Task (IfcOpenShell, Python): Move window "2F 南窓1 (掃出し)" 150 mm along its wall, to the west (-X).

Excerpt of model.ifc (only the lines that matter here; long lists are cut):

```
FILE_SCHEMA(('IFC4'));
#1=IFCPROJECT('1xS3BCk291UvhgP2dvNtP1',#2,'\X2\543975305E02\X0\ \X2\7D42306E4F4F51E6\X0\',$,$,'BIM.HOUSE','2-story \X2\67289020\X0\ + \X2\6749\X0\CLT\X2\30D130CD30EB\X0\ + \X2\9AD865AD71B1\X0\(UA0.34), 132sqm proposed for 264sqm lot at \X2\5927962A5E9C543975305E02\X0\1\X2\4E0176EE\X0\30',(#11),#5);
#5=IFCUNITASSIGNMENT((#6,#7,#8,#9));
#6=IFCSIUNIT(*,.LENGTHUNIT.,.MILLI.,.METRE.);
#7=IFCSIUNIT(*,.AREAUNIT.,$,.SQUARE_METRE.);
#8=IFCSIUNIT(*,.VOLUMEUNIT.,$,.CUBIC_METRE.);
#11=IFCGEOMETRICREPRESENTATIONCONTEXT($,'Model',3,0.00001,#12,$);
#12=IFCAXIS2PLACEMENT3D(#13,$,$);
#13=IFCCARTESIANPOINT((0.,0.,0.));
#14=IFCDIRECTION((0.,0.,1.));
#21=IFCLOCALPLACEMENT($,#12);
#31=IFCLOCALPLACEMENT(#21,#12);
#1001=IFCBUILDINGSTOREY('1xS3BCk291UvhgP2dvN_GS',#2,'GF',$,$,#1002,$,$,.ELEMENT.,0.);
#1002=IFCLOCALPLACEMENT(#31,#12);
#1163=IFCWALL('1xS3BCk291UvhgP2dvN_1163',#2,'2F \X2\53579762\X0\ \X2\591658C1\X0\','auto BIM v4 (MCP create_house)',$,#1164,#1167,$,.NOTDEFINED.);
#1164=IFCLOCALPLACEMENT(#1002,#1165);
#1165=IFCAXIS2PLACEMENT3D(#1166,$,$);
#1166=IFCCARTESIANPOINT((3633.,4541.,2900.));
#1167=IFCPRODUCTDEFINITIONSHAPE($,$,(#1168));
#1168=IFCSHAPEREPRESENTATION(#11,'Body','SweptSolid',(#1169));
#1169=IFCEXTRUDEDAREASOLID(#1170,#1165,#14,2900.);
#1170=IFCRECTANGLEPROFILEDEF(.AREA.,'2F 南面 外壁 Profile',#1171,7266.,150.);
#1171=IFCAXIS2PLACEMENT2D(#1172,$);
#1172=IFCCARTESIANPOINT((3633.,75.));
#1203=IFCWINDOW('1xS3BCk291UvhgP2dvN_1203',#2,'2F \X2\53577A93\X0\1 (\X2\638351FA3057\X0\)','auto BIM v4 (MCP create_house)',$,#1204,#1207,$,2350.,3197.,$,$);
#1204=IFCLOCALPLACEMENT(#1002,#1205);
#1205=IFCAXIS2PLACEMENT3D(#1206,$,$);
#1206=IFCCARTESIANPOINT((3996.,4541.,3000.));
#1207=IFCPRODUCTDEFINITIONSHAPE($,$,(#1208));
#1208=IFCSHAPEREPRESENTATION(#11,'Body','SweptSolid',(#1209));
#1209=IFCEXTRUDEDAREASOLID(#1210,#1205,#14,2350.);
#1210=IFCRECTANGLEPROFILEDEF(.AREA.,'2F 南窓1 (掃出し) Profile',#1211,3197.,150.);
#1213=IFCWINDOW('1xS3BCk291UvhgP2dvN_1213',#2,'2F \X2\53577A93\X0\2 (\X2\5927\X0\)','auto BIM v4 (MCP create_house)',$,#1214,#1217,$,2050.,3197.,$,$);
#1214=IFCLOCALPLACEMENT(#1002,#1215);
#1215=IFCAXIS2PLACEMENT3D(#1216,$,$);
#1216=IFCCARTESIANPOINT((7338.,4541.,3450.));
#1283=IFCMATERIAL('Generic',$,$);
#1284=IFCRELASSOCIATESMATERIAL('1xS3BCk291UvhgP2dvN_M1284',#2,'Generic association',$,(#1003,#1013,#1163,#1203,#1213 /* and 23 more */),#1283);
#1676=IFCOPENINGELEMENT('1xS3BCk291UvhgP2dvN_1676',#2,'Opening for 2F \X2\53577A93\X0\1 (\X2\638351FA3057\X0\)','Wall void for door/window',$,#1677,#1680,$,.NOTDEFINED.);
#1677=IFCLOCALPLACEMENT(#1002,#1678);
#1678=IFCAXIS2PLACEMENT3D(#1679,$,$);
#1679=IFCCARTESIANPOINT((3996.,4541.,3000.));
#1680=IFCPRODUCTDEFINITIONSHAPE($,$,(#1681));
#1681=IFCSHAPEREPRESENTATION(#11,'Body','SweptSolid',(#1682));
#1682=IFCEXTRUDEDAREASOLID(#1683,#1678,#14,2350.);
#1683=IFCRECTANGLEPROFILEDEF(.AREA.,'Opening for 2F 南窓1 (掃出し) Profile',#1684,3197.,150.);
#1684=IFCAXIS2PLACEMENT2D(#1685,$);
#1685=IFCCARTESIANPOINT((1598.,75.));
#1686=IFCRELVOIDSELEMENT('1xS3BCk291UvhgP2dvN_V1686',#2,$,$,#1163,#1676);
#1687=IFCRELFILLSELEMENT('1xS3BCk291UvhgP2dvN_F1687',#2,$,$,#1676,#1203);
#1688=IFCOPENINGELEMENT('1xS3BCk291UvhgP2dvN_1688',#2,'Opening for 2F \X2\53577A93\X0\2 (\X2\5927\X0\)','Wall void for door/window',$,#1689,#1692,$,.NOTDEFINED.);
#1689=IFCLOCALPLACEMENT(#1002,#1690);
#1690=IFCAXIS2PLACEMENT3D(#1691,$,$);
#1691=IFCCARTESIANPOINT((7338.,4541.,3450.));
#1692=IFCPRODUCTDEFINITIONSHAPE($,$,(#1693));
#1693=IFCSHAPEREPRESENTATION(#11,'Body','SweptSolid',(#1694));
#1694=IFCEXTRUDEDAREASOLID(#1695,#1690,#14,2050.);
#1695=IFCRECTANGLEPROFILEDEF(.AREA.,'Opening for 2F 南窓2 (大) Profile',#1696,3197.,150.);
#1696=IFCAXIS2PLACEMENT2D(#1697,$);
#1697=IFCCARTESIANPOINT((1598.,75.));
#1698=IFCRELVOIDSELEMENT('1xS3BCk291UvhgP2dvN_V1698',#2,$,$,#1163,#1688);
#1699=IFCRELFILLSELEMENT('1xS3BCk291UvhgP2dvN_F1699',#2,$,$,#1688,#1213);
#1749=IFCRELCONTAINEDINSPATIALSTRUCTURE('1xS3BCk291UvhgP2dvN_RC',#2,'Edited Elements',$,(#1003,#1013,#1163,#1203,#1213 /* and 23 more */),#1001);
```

```python
import ifcopenshell
import ifcopenshell.api.geometry
import ifcopenshell.util.placement
import ifcopenshell.util.unit

model = ifcopenshell.open("model.ifc")
unit_scale = ifcopenshell.util.unit.calculate_unit_scale(model)

window = model.by_guid("1xS3BCk291UvhgP2dvN_1203")
opening = window.FillsVoids[0].RelatingOpeningElement
wall = opening.VoidsElements[0].RelatingBuildingElement

wall_matrix = ifcopenshell.util.placement.get_local_placement(wall.ObjectPlacement)
shift = wall_matrix[:3, 0] * -0.15 / unit_scale
before = ifcopenshell.util.placement.get_local_placement(window.ObjectPlacement)[:3, 3].copy()

# The window is not placed relative to its opening, so move both.
for product in (opening, window):
    matrix = ifcopenshell.util.placement.get_local_placement(product.ObjectPlacement)
    matrix[:3, 3] += shift
    ifcopenshell.api.geometry.edit_object_placement(model, product=product, matrix=matrix, is_si=False)

after = ifcopenshell.util.placement.get_local_placement(window.ObjectPlacement)[:3, 3]
print("window moved by", (after - before).round(3) + 0.0)

model.write("model_updated.ifc")
```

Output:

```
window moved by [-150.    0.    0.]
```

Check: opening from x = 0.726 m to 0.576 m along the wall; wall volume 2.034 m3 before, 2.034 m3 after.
